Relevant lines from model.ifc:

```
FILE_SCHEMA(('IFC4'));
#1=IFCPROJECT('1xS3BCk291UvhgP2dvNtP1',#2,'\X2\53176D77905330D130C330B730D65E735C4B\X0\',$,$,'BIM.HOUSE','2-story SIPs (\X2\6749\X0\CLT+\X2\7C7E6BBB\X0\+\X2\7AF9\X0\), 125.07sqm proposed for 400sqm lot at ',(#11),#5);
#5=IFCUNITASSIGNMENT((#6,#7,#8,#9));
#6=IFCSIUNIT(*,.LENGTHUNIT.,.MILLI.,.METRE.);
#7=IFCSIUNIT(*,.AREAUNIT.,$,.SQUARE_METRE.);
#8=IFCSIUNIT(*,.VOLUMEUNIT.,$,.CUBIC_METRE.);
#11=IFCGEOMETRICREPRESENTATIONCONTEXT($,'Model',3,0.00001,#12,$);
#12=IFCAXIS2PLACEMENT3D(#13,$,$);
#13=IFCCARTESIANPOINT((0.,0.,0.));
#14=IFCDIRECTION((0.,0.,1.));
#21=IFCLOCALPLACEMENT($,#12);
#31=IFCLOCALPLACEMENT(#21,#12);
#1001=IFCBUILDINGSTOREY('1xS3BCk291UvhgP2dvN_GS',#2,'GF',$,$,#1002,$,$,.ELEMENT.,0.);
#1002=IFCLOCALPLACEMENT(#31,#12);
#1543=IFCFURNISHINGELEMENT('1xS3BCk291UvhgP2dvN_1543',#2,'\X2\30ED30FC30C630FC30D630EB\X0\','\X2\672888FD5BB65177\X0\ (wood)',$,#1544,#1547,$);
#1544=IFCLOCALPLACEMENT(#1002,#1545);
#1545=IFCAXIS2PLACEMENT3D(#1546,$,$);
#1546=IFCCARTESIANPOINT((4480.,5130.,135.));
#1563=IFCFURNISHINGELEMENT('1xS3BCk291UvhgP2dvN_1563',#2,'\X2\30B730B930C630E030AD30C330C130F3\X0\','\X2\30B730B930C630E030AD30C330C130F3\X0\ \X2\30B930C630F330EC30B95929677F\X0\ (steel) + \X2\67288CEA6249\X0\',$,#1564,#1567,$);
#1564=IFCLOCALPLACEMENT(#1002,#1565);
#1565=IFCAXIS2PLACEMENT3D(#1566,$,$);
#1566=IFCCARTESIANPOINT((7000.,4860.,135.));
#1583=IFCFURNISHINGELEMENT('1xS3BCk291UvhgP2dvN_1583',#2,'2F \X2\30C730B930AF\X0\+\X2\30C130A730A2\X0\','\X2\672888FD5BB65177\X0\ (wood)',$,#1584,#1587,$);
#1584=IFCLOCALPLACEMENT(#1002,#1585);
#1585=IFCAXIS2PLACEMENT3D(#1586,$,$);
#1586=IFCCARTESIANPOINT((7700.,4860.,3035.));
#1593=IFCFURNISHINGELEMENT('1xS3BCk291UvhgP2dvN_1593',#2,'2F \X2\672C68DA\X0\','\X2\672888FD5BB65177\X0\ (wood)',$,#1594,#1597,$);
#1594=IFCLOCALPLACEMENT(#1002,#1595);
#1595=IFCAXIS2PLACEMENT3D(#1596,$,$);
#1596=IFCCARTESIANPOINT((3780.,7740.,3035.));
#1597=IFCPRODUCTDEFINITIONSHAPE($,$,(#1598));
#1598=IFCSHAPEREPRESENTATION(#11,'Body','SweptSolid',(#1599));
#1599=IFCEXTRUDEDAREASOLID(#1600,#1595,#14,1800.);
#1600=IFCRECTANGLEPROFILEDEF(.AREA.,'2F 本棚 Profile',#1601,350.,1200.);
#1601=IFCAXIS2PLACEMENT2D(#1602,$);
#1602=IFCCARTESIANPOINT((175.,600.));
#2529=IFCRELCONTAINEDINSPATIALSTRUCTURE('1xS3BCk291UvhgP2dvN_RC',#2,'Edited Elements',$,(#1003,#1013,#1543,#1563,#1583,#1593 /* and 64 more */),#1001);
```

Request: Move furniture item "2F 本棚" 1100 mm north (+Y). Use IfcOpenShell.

```python
import ifcopenshell
import ifcopenshell.api.geometry
import ifcopenshell.util.placement
import ifcopenshell.util.unit

model = ifcopenshell.open("model.ifc")
unit_scale = ifcopenshell.util.unit.calculate_unit_scale(model)

item = model.by_guid("1xS3BCk291UvhgP2dvN_1593")
matrix = ifcopenshell.util.placement.get_local_placement(item.ObjectPlacement)
matrix[1, 3] += 1.1 / unit_scale
ifcopenshell.api.geometry.edit_object_placement(model, product=item, matrix=matrix, is_si=False)

print(ifcopenshell.util.placement.get_local_placement(item.ObjectPlacement).round(3) + 0.0)

model.write("model_v2.ifc")
```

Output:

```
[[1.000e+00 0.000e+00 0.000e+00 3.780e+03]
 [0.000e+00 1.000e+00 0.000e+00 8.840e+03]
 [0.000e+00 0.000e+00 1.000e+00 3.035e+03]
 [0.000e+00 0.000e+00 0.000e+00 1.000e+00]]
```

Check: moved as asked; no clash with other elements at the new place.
